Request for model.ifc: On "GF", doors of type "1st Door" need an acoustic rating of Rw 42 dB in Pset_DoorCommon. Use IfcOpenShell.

First a look at what the model holds.

```python
import ifcopenshell
import ifcopenshell.util.element

model = ifcopenshell.open("model.ifc")
print(model.schema)
storey = next(s for s in model.by_type("IfcBuildingStorey") if s.Name == "GF")
doors = [e for e in ifcopenshell.util.element.get_decomposition(storey) if e.is_a("IfcDoor")]
seen = {}
for e in doors:
    element_type = ifcopenshell.util.element.get_type(e)
    key = (element_type.Name if element_type != e and element_type else None, ifcopenshell.util.element.get_pset(e, "Pset_DoorCommon", "AcousticRating"))
    seen[key] = seen.get(key, 0) + 1
for (name, value), count in sorted(seen.items(), key=str):
    print(count, "x", name, "|", value)
```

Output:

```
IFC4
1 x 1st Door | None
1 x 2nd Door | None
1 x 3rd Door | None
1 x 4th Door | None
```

```python
import ifcopenshell
import ifcopenshell.api.pset
import ifcopenshell.util.element

model = ifcopenshell.open("model.ifc")

storey = next(s for s in model.by_type("IfcBuildingStorey") if s.Name == "GF")
doors = [e for e in ifcopenshell.util.element.get_decomposition(storey) if e.is_a("IfcDoor")]

count = 0
for e in doors:
    element_type = ifcopenshell.util.element.get_type(e)
    if element_type in (None, e) or element_type.Name != "1st Door":
        continue
    # add_pset returns the element's existing set when there is one.
    pset = ifcopenshell.api.pset.add_pset(model, product=e, name="Pset_DoorCommon")
    ifcopenshell.api.pset.edit_pset(model, pset=pset, properties={"AcousticRating": "Rw 42 dB"})
    count += 1

print(count, "doors updated")

model.write("model_rev.ifc")
```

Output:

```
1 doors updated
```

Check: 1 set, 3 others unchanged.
